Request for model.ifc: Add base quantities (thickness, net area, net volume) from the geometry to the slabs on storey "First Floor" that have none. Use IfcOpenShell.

First a look at what the model holds.

```python
import ifcopenshell
import ifcopenshell.util.element
import ifcopenshell.util.unit

model = ifcopenshell.open("model.ifc")
print(model.schema)
for unit_type in ("LENGTHUNIT", "AREAUNIT", "VOLUMEUNIT"):
    print(unit_type, ifcopenshell.util.unit.calculate_unit_scale(model, unit_type))
storey = next(s for s in model.by_type("IfcBuildingStorey") if s.Name == "First Floor")
slabs = [e for e in ifcopenshell.util.element.get_decomposition(storey) if e.is_a("IfcSlab")]
for e in sorted(slabs, key=lambda e: e.id()):
    print(e.id(), e.is_a(), e.Name, list(ifcopenshell.util.element.get_psets(e, qtos_only=True)), sep=" | ")
```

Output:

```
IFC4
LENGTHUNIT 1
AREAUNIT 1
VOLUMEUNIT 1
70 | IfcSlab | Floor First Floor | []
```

```python
import ifcopenshell
import ifcopenshell.api.pset
import ifcopenshell.geom
import ifcopenshell.util.element
import ifcopenshell.util.shape
import ifcopenshell.util.unit

model = ifcopenshell.open("model.ifc")
unit_scale = ifcopenshell.util.unit.calculate_unit_scale(model)
area_scale = ifcopenshell.util.unit.calculate_unit_scale(model, "AREAUNIT")
volume_scale = ifcopenshell.util.unit.calculate_unit_scale(model, "VOLUMEUNIT")
settings = ifcopenshell.geom.settings()

storey = next(s for s in model.by_type("IfcBuildingStorey") if s.Name == "First Floor")
slabs = [e for e in ifcopenshell.util.element.get_decomposition(storey) if e.is_a("IfcSlab")]

for e in sorted(slabs, key=lambda e: e.id()):
    if ifcopenshell.util.element.get_psets(e, qtos_only=True, should_inherit=False):
        continue
    # Geometry comes back in metres, in the element's own axes.
    shape = ifcopenshell.geom.create_shape(settings, e)
    values = {
        "Width": ifcopenshell.util.shape.get_z(shape.geometry) / unit_scale,
        "NetArea": ifcopenshell.util.shape.get_footprint_area(shape.geometry) / area_scale,
        "NetVolume": ifcopenshell.util.shape.get_volume(shape.geometry) / volume_scale,
    }
    qto = ifcopenshell.api.pset.add_qto(model, product=e, name="Qto_SlabBaseQuantities")
    ifcopenshell.api.pset.edit_qto(model, qto=qto, properties=values)
    print(e.id(), {k: round(v, 3) for k, v in values.items()})

model.write("model_v2.ifc")
```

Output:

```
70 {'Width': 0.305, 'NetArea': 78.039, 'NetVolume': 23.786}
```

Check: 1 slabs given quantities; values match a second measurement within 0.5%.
